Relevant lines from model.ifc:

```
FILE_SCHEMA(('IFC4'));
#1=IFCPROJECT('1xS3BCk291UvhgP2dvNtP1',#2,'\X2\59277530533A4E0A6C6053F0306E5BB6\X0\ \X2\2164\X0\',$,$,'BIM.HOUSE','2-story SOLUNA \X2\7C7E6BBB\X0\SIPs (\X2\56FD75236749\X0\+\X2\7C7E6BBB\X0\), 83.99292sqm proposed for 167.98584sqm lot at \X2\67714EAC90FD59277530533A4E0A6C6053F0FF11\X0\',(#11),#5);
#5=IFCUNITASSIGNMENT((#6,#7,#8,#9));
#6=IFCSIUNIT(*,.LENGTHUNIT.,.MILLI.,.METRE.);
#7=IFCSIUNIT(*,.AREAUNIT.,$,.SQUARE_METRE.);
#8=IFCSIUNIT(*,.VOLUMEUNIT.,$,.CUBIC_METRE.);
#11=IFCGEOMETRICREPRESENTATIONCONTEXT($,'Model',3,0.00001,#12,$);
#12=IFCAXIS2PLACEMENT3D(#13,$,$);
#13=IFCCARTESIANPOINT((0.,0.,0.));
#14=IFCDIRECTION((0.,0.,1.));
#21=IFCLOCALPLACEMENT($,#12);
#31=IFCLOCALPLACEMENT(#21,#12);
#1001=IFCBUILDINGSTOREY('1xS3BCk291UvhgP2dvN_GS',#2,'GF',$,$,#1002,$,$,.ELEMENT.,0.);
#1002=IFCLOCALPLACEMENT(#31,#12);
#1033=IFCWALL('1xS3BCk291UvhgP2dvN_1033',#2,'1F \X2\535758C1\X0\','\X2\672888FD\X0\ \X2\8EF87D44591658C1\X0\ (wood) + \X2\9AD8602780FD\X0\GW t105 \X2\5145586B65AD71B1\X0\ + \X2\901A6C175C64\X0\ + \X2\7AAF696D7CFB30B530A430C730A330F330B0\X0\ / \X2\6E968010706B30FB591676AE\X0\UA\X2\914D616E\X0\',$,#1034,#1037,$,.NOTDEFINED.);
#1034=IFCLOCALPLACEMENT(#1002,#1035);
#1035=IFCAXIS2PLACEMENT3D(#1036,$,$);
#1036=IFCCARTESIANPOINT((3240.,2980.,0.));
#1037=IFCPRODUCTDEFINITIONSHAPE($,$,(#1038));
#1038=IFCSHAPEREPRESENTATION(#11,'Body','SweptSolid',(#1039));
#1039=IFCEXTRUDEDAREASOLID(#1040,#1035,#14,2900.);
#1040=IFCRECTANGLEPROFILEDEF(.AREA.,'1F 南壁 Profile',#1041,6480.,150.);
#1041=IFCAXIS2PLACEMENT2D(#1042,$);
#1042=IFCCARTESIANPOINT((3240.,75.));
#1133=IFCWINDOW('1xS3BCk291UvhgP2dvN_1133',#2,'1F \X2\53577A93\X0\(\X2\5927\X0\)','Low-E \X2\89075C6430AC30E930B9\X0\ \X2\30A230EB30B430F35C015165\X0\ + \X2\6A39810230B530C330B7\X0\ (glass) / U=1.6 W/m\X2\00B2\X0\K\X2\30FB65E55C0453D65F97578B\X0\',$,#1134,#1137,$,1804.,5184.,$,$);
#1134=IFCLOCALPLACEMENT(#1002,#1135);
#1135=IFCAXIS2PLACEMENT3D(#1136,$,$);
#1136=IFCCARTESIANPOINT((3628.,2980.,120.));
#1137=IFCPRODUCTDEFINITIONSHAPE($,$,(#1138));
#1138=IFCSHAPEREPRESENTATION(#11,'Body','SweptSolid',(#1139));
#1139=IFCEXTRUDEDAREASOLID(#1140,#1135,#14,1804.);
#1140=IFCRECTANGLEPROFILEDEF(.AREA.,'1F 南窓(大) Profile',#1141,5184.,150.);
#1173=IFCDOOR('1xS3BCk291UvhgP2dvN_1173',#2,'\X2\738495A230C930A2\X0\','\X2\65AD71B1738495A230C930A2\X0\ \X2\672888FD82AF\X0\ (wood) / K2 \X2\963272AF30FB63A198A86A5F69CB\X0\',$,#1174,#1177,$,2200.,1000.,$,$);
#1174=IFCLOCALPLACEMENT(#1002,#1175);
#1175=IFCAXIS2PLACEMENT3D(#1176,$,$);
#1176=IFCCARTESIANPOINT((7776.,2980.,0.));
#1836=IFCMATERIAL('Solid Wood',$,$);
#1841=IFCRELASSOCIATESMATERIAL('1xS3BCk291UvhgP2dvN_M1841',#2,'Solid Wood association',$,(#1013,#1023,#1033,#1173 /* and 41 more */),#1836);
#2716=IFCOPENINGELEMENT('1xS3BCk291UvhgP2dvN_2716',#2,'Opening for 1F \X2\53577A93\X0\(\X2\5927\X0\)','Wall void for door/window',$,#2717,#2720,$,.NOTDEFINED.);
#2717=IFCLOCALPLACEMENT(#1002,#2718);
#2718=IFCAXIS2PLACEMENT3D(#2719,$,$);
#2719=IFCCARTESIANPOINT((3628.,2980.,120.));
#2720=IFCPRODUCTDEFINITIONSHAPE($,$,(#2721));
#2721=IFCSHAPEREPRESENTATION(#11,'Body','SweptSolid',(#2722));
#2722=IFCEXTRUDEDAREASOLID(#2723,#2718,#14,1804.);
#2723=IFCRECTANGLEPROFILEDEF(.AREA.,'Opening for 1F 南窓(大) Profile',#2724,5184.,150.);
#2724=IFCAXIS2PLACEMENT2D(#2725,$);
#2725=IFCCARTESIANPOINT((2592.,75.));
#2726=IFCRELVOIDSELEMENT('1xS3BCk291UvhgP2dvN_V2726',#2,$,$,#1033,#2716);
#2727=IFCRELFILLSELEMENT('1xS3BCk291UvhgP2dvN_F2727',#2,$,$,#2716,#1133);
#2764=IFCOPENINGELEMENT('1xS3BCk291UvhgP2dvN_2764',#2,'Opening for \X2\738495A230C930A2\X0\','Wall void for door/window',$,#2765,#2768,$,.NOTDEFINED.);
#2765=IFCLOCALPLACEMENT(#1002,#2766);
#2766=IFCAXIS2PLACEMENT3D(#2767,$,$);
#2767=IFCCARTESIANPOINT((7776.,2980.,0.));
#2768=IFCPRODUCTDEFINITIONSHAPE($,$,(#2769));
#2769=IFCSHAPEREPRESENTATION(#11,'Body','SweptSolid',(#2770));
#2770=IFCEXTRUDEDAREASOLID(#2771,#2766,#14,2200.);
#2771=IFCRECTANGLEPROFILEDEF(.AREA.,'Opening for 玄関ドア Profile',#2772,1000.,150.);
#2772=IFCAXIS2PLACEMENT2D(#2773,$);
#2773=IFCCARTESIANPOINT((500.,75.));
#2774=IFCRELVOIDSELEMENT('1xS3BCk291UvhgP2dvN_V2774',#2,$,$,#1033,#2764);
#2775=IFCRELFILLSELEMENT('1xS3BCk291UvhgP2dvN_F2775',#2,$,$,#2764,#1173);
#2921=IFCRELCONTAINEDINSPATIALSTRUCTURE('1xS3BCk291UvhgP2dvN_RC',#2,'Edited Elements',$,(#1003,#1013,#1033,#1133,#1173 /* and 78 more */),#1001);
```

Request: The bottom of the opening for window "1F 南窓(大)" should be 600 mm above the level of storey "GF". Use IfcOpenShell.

```python
import numpy as np
import ifcopenshell
import ifcopenshell.api.geometry
import ifcopenshell.geom
import ifcopenshell.util.element
import ifcopenshell.util.placement
import ifcopenshell.util.shape
import ifcopenshell.util.unit

model = ifcopenshell.open("model.ifc")
unit_scale = ifcopenshell.util.unit.calculate_unit_scale(model)

window = model.by_guid("1xS3BCk291UvhgP2dvN_1133")
opening = window.FillsVoids[0].RelatingOpeningElement
storey = ifcopenshell.util.element.get_container(window, ifc_class="IfcBuildingStorey")
level = ifcopenshell.util.placement.get_local_placement(storey.ObjectPlacement)[2, 3]

# The opening's origin need not be at the sill, so measure its lowest point.
shape = ifcopenshell.geom.create_shape(ifcopenshell.geom.settings(), opening)
bottom = ifcopenshell.util.shape.get_shape_bottom_elevation(shape, shape.geometry) / unit_scale
dz = level + 0.6 / unit_scale - bottom

shift = np.array([0.0, 0.0, dz])
# The window is not placed relative to its opening, so move both.
for product in (opening, window):
    matrix = ifcopenshell.util.placement.get_local_placement(product.ObjectPlacement)
    matrix[:3, 3] += shift
    ifcopenshell.api.geometry.edit_object_placement(model, product=product, matrix=matrix, is_si=False)

print(f"moved by {dz * unit_scale:+.3f} m")

model.write("model_edited.ifc")
```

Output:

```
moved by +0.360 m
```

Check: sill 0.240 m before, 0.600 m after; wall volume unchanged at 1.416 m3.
